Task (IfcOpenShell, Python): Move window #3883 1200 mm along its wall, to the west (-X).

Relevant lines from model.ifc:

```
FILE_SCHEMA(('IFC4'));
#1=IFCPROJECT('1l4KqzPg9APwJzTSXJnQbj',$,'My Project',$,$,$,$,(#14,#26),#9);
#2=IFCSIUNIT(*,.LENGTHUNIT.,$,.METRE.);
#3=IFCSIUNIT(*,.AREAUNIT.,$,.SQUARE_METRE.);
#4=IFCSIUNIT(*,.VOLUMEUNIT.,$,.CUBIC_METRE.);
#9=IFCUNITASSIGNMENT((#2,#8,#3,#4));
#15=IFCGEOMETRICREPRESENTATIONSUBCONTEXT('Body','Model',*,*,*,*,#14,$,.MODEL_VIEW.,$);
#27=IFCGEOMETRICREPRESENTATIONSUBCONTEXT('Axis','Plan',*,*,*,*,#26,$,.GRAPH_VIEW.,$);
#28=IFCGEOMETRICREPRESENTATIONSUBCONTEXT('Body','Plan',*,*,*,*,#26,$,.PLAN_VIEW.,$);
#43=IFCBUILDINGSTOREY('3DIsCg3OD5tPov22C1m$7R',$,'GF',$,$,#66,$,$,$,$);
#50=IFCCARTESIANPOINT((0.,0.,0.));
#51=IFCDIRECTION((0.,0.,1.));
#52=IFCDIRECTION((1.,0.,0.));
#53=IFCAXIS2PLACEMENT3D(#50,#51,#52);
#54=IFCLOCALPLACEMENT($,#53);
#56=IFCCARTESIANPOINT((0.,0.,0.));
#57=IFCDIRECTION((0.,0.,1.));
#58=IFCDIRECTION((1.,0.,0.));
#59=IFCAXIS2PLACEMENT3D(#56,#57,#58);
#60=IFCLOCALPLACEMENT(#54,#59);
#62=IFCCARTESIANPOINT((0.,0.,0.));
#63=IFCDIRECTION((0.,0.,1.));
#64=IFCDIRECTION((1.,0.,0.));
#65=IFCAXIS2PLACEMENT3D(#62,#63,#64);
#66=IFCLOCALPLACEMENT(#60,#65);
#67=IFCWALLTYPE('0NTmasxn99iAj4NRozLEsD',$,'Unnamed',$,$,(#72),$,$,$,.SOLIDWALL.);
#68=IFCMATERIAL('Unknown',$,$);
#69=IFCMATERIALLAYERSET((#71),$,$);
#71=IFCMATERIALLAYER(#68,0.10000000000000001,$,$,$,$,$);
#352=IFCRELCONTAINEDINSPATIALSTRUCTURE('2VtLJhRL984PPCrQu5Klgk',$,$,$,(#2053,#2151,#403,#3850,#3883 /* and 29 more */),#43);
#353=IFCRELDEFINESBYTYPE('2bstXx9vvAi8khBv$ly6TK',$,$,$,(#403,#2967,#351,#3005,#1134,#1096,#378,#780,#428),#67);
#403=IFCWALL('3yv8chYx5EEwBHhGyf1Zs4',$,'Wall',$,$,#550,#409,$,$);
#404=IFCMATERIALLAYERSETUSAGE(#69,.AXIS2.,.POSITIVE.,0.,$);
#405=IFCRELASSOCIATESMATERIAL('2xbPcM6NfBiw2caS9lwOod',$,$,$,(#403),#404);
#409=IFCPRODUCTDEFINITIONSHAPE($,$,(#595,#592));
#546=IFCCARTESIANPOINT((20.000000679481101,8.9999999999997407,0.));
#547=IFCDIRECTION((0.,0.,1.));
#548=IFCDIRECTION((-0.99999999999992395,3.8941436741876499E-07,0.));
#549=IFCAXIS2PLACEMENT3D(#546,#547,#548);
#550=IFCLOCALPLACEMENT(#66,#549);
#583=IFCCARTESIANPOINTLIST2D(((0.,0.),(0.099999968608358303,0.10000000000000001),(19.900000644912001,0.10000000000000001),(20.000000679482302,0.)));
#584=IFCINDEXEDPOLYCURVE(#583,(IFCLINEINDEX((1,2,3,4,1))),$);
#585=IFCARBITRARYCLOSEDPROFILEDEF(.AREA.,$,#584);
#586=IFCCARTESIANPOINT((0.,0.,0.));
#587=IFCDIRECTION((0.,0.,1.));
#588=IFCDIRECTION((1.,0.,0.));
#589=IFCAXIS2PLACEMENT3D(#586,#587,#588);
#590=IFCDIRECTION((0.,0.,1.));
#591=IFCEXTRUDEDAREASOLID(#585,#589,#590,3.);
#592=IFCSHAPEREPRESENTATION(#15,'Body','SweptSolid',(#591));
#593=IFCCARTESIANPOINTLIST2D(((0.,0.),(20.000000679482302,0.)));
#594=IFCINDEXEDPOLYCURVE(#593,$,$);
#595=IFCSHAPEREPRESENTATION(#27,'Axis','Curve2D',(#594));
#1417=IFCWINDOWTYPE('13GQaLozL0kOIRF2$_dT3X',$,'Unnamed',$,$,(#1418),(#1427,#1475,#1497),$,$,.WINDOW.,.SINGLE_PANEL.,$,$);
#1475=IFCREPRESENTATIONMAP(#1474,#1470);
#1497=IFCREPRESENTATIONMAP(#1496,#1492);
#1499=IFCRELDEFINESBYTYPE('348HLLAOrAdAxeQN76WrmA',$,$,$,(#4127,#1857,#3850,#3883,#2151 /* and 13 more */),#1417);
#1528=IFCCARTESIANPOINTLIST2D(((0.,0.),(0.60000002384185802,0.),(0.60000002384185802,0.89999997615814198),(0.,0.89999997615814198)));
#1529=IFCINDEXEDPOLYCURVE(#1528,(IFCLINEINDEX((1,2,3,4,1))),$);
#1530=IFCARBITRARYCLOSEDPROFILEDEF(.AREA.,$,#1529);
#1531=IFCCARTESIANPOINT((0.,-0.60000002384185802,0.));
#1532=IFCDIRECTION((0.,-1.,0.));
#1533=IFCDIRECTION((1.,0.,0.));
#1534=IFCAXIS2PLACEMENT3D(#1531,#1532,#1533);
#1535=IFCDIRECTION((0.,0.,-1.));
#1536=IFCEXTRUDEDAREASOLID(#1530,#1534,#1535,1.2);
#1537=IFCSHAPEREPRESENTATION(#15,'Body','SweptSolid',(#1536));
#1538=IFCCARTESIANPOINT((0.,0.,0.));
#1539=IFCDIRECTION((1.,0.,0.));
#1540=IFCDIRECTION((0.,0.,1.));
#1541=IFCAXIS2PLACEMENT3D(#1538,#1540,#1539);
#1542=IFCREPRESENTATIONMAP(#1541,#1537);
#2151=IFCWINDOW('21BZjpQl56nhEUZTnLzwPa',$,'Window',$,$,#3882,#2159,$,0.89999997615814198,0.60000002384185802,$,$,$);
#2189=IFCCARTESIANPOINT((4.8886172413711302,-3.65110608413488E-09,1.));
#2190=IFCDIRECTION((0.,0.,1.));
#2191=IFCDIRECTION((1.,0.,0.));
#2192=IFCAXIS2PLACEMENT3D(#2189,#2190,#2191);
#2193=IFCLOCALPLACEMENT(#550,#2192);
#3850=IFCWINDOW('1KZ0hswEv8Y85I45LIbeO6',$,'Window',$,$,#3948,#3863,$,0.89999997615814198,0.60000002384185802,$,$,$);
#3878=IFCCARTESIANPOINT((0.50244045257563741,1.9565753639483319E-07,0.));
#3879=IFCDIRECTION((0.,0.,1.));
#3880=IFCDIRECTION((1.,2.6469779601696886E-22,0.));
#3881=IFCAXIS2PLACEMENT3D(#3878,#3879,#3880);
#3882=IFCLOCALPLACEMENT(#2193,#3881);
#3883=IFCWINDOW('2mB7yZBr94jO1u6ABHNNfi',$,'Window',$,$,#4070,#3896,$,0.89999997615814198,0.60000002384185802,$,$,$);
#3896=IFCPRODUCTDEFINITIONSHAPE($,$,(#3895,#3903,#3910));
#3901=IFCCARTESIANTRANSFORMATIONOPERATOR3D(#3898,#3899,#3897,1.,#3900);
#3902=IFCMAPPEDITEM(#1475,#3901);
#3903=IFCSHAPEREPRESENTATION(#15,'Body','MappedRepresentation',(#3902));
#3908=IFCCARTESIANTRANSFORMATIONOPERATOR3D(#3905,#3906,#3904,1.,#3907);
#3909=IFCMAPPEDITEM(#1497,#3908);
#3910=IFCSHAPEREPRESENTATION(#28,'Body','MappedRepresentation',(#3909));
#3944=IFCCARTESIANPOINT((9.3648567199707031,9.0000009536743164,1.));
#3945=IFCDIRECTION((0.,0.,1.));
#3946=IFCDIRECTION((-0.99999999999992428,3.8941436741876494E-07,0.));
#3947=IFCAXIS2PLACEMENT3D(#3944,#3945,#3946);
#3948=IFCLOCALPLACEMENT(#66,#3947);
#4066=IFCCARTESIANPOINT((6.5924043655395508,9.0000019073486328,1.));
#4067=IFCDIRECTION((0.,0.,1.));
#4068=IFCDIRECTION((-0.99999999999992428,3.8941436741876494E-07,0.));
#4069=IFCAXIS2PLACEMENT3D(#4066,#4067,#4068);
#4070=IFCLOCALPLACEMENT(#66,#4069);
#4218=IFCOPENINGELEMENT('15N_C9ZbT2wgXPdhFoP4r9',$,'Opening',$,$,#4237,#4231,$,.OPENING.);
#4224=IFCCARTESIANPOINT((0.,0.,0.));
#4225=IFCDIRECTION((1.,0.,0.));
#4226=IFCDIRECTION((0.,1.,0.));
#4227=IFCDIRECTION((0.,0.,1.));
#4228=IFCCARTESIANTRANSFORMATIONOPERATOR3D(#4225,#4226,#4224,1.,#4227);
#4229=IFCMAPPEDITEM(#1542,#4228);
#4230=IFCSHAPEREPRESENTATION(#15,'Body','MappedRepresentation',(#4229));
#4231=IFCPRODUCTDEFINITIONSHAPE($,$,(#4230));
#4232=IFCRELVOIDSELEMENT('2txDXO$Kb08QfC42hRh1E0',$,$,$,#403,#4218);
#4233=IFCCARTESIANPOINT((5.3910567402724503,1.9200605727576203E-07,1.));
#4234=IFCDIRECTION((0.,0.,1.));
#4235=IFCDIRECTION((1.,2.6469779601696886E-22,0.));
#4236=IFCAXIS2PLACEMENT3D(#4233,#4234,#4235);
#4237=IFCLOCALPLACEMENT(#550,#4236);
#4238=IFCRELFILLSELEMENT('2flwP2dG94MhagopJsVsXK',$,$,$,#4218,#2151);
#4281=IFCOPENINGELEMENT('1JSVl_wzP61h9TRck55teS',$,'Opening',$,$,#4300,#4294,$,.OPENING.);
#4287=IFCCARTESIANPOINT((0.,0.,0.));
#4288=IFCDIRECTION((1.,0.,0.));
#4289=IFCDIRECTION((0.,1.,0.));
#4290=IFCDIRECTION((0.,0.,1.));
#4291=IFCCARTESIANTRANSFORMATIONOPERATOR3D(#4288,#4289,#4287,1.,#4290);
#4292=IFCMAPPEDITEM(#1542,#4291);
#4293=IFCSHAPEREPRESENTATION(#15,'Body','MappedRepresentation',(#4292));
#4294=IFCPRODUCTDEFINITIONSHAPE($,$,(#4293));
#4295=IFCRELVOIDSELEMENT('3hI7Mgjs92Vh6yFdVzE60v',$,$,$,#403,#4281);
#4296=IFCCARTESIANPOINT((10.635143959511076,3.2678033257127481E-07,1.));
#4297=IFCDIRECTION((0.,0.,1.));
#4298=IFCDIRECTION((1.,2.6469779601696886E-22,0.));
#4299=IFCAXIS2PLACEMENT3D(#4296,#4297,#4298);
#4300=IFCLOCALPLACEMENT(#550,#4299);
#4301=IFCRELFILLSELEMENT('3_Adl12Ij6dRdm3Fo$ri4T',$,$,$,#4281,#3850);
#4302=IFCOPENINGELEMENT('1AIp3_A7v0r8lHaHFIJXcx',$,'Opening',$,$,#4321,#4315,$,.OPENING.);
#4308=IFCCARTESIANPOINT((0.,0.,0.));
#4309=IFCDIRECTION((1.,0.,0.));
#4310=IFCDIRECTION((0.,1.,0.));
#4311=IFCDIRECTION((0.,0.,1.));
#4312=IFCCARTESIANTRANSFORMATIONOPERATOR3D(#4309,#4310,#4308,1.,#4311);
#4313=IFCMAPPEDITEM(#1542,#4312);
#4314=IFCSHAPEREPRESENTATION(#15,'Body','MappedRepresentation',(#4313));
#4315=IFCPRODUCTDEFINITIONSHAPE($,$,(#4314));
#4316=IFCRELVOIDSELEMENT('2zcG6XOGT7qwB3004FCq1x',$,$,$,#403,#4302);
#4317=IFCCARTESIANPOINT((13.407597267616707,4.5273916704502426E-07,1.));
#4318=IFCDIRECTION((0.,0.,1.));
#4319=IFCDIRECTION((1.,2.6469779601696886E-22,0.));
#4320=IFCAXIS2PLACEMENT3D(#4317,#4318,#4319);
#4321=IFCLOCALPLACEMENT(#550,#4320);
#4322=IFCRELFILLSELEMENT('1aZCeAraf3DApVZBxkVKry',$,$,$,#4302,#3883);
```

```python
import ifcopenshell
import ifcopenshell.api.geometry
import ifcopenshell.util.placement
import ifcopenshell.util.unit

model = ifcopenshell.open("model.ifc")
unit_scale = ifcopenshell.util.unit.calculate_unit_scale(model)

window = model.by_id(3883)
opening = window.FillsVoids[0].RelatingOpeningElement
wall = opening.VoidsElements[0].RelatingBuildingElement

wall_matrix = ifcopenshell.util.placement.get_local_placement(wall.ObjectPlacement)
shift = wall_matrix[:3, 0] * 1.2 / unit_scale
before = ifcopenshell.util.placement.get_local_placement(window.ObjectPlacement)[:3, 3].copy()

# The window is not placed relative to its opening, so move both.
for product in (opening, window):
    matrix = ifcopenshell.util.placement.get_local_placement(product.ObjectPlacement)
    matrix[:3, 3] += shift
    ifcopenshell.api.geometry.edit_object_placement(model, product=product, matrix=matrix, is_si=False)

after = ifcopenshell.util.placement.get_local_placement(window.ObjectPlacement)[:3, 3]
print("window moved by", (after - before).round(3) + 0.0)

model.write("model_edited.ifc")
```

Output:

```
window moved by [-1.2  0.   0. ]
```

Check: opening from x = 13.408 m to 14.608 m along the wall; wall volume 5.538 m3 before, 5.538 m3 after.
